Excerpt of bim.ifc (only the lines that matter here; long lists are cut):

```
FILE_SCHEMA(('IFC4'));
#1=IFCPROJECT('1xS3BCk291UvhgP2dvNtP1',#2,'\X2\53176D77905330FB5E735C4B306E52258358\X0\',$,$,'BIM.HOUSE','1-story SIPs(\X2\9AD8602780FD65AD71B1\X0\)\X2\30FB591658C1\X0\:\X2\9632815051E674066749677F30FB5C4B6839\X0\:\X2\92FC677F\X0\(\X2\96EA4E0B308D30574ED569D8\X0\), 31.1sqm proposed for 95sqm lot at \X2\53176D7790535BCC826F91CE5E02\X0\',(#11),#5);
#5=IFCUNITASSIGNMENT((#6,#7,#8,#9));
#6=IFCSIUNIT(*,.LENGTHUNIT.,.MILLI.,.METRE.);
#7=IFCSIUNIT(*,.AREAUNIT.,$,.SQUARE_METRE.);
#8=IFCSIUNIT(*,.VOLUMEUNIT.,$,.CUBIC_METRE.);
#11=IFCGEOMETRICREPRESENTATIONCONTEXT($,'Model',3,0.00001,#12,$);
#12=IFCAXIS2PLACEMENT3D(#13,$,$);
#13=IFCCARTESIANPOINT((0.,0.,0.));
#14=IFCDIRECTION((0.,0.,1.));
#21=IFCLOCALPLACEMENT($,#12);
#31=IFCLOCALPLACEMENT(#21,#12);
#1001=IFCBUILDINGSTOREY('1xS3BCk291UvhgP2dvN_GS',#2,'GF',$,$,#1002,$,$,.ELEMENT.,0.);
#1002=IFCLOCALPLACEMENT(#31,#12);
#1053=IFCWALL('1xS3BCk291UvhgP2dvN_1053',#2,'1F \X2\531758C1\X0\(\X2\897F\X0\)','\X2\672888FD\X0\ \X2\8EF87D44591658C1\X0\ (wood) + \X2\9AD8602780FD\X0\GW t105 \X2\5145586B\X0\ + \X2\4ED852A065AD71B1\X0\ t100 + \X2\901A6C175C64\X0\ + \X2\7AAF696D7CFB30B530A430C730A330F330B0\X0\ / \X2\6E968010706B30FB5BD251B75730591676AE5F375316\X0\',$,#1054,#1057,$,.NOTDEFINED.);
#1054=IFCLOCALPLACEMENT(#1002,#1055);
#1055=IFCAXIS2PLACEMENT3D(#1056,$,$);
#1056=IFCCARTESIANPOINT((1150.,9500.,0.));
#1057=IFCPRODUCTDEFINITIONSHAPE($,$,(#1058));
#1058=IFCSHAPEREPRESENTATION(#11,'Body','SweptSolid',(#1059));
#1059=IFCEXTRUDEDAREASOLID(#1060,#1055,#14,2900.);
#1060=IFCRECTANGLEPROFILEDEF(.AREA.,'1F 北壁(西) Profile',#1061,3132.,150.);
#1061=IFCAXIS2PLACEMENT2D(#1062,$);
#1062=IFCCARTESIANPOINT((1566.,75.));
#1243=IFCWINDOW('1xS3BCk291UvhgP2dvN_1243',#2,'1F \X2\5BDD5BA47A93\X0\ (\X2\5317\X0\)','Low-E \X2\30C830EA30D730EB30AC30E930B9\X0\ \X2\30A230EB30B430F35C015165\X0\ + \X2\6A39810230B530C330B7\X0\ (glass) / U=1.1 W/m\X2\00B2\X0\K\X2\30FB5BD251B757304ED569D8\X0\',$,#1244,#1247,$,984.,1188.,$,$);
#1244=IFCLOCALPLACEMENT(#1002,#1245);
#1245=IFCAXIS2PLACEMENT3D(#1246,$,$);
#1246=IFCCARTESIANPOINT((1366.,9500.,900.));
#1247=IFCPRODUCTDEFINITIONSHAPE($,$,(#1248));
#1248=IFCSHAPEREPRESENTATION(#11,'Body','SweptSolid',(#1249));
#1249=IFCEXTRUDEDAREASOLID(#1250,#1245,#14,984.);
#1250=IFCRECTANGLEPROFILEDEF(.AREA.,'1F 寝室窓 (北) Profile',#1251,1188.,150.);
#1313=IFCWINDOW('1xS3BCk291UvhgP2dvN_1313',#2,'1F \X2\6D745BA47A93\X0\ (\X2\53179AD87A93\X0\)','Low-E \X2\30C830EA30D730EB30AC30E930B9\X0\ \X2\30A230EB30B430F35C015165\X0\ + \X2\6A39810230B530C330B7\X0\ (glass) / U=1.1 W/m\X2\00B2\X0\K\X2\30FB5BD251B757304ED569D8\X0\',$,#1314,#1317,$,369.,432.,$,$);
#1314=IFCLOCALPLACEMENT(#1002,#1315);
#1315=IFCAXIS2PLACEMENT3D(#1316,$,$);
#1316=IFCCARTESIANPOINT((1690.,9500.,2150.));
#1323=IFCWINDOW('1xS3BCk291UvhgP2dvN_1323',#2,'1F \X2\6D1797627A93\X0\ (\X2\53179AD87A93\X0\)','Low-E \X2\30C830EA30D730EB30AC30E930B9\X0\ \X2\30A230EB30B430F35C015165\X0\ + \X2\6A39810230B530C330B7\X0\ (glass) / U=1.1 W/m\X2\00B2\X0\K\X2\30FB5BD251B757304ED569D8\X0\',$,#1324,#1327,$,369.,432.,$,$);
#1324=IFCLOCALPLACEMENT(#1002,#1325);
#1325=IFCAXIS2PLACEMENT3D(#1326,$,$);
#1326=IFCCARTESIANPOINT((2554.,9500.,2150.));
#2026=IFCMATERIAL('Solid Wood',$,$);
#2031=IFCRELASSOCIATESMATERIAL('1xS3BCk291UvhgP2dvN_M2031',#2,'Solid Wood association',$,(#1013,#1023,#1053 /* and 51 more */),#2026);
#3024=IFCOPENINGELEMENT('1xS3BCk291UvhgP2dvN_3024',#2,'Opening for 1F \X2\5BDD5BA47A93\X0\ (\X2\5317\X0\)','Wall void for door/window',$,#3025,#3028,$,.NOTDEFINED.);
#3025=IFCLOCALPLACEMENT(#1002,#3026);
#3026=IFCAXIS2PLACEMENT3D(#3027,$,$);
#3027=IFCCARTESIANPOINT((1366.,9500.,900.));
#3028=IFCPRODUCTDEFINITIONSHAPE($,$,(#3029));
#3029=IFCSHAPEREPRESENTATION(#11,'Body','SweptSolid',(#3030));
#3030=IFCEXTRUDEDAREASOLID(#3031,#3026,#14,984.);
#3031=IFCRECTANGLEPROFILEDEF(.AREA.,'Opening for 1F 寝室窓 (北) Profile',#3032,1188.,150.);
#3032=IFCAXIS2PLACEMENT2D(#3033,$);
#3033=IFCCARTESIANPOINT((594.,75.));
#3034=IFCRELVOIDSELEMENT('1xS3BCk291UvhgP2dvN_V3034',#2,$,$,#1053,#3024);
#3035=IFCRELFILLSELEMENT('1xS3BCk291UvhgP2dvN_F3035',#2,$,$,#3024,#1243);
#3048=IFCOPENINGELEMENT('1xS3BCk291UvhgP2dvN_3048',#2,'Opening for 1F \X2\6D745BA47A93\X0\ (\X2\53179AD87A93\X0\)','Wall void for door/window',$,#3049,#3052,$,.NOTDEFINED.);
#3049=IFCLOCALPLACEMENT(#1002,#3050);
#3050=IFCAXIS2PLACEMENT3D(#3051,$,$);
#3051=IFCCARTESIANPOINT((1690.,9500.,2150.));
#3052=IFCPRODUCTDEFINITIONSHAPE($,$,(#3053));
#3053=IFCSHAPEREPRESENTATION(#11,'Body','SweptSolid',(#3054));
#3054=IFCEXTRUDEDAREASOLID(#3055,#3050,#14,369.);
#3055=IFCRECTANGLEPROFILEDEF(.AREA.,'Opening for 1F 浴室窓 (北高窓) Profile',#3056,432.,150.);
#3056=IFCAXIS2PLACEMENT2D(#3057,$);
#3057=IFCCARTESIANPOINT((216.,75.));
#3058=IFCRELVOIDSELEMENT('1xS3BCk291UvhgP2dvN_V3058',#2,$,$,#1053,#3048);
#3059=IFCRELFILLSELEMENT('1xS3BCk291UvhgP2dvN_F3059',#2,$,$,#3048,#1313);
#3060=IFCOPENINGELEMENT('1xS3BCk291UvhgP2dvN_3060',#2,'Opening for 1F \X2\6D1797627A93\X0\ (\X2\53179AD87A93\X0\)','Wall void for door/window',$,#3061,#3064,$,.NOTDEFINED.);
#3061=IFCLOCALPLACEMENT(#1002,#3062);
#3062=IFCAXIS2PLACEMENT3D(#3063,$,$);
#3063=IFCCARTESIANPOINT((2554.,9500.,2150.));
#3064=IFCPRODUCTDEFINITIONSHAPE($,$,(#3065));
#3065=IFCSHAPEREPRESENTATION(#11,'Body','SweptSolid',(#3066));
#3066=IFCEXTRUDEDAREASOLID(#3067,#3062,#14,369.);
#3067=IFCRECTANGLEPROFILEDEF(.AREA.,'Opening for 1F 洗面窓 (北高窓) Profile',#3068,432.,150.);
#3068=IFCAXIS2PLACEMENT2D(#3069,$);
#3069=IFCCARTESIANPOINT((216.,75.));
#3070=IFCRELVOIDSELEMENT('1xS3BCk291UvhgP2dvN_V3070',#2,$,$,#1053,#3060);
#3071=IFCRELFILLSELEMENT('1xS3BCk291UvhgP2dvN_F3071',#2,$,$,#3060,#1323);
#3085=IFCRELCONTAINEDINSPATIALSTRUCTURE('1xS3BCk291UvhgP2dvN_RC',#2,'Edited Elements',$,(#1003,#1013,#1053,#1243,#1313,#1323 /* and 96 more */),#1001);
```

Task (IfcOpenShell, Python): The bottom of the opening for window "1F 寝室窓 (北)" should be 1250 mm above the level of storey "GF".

```python
import numpy as np
import ifcopenshell
import ifcopenshell.api.geometry
import ifcopenshell.geom
import ifcopenshell.util.element
import ifcopenshell.util.placement
import ifcopenshell.util.shape
import ifcopenshell.util.unit

model = ifcopenshell.open("bim.ifc")
unit_scale = ifcopenshell.util.unit.calculate_unit_scale(model)

window = model.by_guid("1xS3BCk291UvhgP2dvN_1243")
opening = window.FillsVoids[0].RelatingOpeningElement
storey = ifcopenshell.util.element.get_container(window, ifc_class="IfcBuildingStorey")
level = ifcopenshell.util.placement.get_local_placement(storey.ObjectPlacement)[2, 3]

# The opening's origin need not be at the sill, so measure its lowest point.
shape = ifcopenshell.geom.create_shape(ifcopenshell.geom.settings(), opening)
bottom = ifcopenshell.util.shape.get_shape_bottom_elevation(shape, shape.geometry) / unit_scale
dz = level + 1.25 / unit_scale - bottom

shift = np.array([0.0, 0.0, dz])
# The window is not placed relative to its opening, so move both.
for product in (opening, window):
    matrix = ifcopenshell.util.placement.get_local_placement(product.ObjectPlacement)
    matrix[:3, 3] += shift
    ifcopenshell.api.geometry.edit_object_placement(model, product=product, matrix=matrix, is_si=False)

print(f"moved by {dz * unit_scale:+.3f} m")

model.write("bim_rev.ifc")
```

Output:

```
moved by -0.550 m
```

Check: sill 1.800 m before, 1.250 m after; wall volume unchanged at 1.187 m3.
